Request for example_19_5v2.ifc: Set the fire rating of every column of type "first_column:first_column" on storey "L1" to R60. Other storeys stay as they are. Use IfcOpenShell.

First a look at what the model holds.

```python
import ifcopenshell
import ifcopenshell.util.element

model = ifcopenshell.open("example_19_5v2.ifc")
print(model.schema)
storey = next(s for s in model.by_type("IfcBuildingStorey") if s.Name == "L1")
columns = [e for e in ifcopenshell.util.element.get_decomposition(storey) if e.is_a("IfcColumn")]
seen = {}
for e in columns:
    element_type = ifcopenshell.util.element.get_type(e)
    key = (element_type.Name if element_type != e and element_type else None, ifcopenshell.util.element.get_pset(e, "Pset_ColumnCommon", "FireRating"))
    seen[key] = seen.get(key, 0) + 1
for (name, value), count in sorted(seen.items(), key=str):
    print(count, "x", name, "|", value)
```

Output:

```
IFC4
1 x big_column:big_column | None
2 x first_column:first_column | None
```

```python
import ifcopenshell
import ifcopenshell.api.pset
import ifcopenshell.util.element

model = ifcopenshell.open("example_19_5v2.ifc")

storey = next(s for s in model.by_type("IfcBuildingStorey") if s.Name == "L1")
columns = [e for e in ifcopenshell.util.element.get_decomposition(storey) if e.is_a("IfcColumn")]

count = 0
for e in columns:
    element_type = ifcopenshell.util.element.get_type(e)
    if element_type in (None, e) or element_type.Name != "first_column:first_column":
        continue
    # add_pset returns the element's existing set when there is one.
    pset = ifcopenshell.api.pset.add_pset(model, product=e, name="Pset_ColumnCommon")
    ifcopenshell.api.pset.edit_pset(model, pset=pset, properties={"FireRating": "R60"})
    count += 1

print(count, "columns updated")

model.write("example_19_5v2_v2.ifc")
```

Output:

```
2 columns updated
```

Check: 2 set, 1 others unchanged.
